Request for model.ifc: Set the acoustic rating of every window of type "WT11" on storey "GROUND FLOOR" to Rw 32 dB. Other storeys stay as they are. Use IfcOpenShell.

First a look at what the model holds.

```python
import ifcopenshell
import ifcopenshell.util.element

model = ifcopenshell.open("model.ifc")
print(model.schema)
storey = next(s for s in model.by_type("IfcBuildingStorey") if s.Name == "GROUND FLOOR")
windows = [e for e in ifcopenshell.util.element.get_decomposition(storey) if e.is_a("IfcWindow")]
seen = {}
for e in windows:
    element_type = ifcopenshell.util.element.get_type(e)
    key = (element_type.Name if element_type != e and element_type else None, ifcopenshell.util.element.get_pset(e, "Pset_WindowCommon", "AcousticRating"))
    seen[key] = seen.get(key, 0) + 1
for (name, value), count in sorted(seen.items(), key=str):
    print(count, "x", name, "|", value)
```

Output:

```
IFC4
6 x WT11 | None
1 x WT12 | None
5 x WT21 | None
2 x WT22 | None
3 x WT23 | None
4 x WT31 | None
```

```python
import ifcopenshell
import ifcopenshell.api.pset
import ifcopenshell.util.element

model = ifcopenshell.open("model.ifc")

storey = next(s for s in model.by_type("IfcBuildingStorey") if s.Name == "GROUND FLOOR")
windows = [e for e in ifcopenshell.util.element.get_decomposition(storey) if e.is_a("IfcWindow")]

count = 0
for e in windows:
    element_type = ifcopenshell.util.element.get_type(e)
    if element_type in (None, e) or element_type.Name != "WT11":
        continue
    # add_pset returns the element's existing set when there is one.
    pset = ifcopenshell.api.pset.add_pset(model, product=e, name="Pset_WindowCommon")
    ifcopenshell.api.pset.edit_pset(model, pset=pset, properties={"AcousticRating": "Rw 32 dB"})
    count += 1

print(count, "windows updated")

model.write("model_v2.ifc")
```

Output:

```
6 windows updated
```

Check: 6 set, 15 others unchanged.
